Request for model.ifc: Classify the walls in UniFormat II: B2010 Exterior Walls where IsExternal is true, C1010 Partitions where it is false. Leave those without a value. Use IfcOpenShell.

First a look at what the model holds.

```python
import ifcopenshell
import ifcopenshell.util.element

model = ifcopenshell.open("model.ifc")
print(model.schema)
print("classifications:", [c.Name for c in model.by_type("IfcClassification")])
values = [ifcopenshell.util.element.get_pset(e, "Pset_WallCommon", "IsExternal") for e in model.by_type("IfcWall")]
for value in (True, False, None):
    print("IsExternal", value, values.count(value))
```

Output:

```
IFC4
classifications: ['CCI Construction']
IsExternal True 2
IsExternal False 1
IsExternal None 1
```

```python
import ifcopenshell
import ifcopenshell.api.classification
import ifcopenshell.util.element

model = ifcopenshell.open("model.ifc")

system = ifcopenshell.api.classification.add_classification(model, classification="UniFormat II")

walls = model.by_type("IfcWall")
external = {e: ifcopenshell.util.element.get_pset(e, "Pset_WallCommon", "IsExternal") for e in walls}
for flag, code, name in ((True, "B2010", "Exterior Walls"), (False, "C1010", "Partitions")):
    products = [e for e in walls if external[e] is flag]
    ifcopenshell.api.classification.add_reference(
        model, products=products, classification=system, identification=code, name=name
    )
    print(code, len(products))

model.write("model_edited.ifc")
```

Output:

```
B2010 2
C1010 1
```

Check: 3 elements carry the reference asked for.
